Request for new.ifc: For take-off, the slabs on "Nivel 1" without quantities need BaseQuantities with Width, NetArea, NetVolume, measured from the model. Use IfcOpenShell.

First a look at what the model holds.

```python
import ifcopenshell
import ifcopenshell.util.element
import ifcopenshell.util.unit

model = ifcopenshell.open("new.ifc")
print(model.schema)
for unit_type in ("LENGTHUNIT", "AREAUNIT", "VOLUMEUNIT"):
    print(unit_type, ifcopenshell.util.unit.calculate_unit_scale(model, unit_type))
storey = next(s for s in model.by_type("IfcBuildingStorey") if s.Name == "Nivel 1")
slabs = [e for e in ifcopenshell.util.element.get_decomposition(storey) if e.is_a("IfcSlab")]
for e in sorted(slabs, key=lambda e: e.id()):
    print(e.id(), e.is_a(), e.Name, list(ifcopenshell.util.element.get_psets(e, qtos_only=True)), sep=" | ")
```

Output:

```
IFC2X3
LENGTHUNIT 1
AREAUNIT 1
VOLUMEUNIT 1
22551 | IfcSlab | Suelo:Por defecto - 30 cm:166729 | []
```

```python
import ifcopenshell
import ifcopenshell.api.pset
import ifcopenshell.geom
import ifcopenshell.util.element
import ifcopenshell.util.shape
import ifcopenshell.util.unit

model = ifcopenshell.open("new.ifc")
unit_scale = ifcopenshell.util.unit.calculate_unit_scale(model)
area_scale = ifcopenshell.util.unit.calculate_unit_scale(model, "AREAUNIT")
volume_scale = ifcopenshell.util.unit.calculate_unit_scale(model, "VOLUMEUNIT")
settings = ifcopenshell.geom.settings()

storey = next(s for s in model.by_type("IfcBuildingStorey") if s.Name == "Nivel 1")
slabs = [e for e in ifcopenshell.util.element.get_decomposition(storey) if e.is_a("IfcSlab")]

for e in sorted(slabs, key=lambda e: e.id()):
    if ifcopenshell.util.element.get_psets(e, qtos_only=True, should_inherit=False):
        continue
    # Geometry comes back in metres, in the element's own axes.
    shape = ifcopenshell.geom.create_shape(settings, e)
    values = {
        "Width": ifcopenshell.util.shape.get_z(shape.geometry) / unit_scale,
        "NetArea": ifcopenshell.util.shape.get_footprint_area(shape.geometry) / area_scale,
        "NetVolume": ifcopenshell.util.shape.get_volume(shape.geometry) / volume_scale,
    }
    qto = ifcopenshell.api.pset.add_qto(model, product=e, name="BaseQuantities")
    ifcopenshell.api.pset.edit_qto(model, qto=qto, properties=values)
    print(e.id(), {k: round(v, 3) for k, v in values.items()})

model.write("new_edited.ifc")
```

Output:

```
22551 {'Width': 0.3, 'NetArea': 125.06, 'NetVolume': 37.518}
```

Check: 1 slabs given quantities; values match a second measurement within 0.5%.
